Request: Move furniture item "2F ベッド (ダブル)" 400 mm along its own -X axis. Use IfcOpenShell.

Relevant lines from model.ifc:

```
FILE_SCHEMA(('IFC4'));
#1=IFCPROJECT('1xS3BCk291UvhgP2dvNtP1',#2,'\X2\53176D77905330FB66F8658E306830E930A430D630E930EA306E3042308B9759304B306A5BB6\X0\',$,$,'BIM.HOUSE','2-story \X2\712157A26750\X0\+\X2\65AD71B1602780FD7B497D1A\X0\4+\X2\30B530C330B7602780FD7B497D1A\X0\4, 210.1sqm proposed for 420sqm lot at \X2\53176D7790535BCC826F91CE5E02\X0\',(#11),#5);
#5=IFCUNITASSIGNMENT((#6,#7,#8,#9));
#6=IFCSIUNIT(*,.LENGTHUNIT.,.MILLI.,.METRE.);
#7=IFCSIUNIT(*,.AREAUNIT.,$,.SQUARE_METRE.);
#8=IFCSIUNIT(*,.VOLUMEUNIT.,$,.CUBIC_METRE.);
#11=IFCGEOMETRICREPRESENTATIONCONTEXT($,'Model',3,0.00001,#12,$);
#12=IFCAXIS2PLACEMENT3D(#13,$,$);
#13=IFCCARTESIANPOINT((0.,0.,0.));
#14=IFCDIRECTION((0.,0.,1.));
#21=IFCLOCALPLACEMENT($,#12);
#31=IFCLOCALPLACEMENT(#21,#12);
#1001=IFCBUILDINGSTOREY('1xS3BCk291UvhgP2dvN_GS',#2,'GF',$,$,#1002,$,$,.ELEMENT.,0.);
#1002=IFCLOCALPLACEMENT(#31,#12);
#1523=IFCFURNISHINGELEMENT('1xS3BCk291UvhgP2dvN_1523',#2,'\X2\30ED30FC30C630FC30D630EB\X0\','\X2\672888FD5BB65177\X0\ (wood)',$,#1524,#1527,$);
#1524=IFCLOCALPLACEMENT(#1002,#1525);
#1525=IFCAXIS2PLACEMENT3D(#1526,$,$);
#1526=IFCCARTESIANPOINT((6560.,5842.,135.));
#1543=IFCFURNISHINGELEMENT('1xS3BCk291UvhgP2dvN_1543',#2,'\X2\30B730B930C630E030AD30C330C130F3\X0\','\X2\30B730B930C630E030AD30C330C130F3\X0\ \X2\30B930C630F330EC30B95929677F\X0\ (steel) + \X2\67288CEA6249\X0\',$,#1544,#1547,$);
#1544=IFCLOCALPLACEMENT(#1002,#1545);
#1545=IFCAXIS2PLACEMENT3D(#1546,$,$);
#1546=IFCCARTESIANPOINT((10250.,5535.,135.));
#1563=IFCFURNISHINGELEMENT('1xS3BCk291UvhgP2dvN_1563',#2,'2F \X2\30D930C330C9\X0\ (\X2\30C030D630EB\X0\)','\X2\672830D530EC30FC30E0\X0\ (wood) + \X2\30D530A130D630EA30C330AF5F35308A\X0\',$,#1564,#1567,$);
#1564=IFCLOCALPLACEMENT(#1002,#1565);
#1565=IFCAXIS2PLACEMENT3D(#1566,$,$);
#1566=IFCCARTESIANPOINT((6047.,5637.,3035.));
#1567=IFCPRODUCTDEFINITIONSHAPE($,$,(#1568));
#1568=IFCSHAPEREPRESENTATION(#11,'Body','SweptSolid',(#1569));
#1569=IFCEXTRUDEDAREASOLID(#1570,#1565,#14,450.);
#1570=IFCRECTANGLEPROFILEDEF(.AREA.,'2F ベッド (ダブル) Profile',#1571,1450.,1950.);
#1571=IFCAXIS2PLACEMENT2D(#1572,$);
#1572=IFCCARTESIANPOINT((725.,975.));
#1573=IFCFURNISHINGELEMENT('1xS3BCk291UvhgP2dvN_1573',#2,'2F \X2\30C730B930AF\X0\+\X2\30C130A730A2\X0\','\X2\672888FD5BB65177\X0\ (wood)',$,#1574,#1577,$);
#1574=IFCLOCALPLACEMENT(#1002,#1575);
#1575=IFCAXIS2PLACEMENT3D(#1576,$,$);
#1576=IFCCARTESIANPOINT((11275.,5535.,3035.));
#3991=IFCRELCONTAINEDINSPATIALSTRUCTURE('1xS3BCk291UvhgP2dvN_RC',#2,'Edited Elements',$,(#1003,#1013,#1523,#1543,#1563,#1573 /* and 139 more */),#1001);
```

```python
import ifcopenshell
import ifcopenshell.api.geometry
import ifcopenshell.util.placement
import ifcopenshell.util.unit

model = ifcopenshell.open("model.ifc")
unit_scale = ifcopenshell.util.unit.calculate_unit_scale(model)

item = model.by_id(1563)
matrix = ifcopenshell.util.placement.get_local_placement(item.ObjectPlacement)
matrix[:3, 3] -= matrix[:3, 0] * 0.4 / unit_scale
ifcopenshell.api.geometry.edit_object_placement(model, product=item, matrix=matrix, is_si=False)

print(ifcopenshell.util.placement.get_local_placement(item.ObjectPlacement).round(3) + 0.0)

model.write("model-out.ifc")
```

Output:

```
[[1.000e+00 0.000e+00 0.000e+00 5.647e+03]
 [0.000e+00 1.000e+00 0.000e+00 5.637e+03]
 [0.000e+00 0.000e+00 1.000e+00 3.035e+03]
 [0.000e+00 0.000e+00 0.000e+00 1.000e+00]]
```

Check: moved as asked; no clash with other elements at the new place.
